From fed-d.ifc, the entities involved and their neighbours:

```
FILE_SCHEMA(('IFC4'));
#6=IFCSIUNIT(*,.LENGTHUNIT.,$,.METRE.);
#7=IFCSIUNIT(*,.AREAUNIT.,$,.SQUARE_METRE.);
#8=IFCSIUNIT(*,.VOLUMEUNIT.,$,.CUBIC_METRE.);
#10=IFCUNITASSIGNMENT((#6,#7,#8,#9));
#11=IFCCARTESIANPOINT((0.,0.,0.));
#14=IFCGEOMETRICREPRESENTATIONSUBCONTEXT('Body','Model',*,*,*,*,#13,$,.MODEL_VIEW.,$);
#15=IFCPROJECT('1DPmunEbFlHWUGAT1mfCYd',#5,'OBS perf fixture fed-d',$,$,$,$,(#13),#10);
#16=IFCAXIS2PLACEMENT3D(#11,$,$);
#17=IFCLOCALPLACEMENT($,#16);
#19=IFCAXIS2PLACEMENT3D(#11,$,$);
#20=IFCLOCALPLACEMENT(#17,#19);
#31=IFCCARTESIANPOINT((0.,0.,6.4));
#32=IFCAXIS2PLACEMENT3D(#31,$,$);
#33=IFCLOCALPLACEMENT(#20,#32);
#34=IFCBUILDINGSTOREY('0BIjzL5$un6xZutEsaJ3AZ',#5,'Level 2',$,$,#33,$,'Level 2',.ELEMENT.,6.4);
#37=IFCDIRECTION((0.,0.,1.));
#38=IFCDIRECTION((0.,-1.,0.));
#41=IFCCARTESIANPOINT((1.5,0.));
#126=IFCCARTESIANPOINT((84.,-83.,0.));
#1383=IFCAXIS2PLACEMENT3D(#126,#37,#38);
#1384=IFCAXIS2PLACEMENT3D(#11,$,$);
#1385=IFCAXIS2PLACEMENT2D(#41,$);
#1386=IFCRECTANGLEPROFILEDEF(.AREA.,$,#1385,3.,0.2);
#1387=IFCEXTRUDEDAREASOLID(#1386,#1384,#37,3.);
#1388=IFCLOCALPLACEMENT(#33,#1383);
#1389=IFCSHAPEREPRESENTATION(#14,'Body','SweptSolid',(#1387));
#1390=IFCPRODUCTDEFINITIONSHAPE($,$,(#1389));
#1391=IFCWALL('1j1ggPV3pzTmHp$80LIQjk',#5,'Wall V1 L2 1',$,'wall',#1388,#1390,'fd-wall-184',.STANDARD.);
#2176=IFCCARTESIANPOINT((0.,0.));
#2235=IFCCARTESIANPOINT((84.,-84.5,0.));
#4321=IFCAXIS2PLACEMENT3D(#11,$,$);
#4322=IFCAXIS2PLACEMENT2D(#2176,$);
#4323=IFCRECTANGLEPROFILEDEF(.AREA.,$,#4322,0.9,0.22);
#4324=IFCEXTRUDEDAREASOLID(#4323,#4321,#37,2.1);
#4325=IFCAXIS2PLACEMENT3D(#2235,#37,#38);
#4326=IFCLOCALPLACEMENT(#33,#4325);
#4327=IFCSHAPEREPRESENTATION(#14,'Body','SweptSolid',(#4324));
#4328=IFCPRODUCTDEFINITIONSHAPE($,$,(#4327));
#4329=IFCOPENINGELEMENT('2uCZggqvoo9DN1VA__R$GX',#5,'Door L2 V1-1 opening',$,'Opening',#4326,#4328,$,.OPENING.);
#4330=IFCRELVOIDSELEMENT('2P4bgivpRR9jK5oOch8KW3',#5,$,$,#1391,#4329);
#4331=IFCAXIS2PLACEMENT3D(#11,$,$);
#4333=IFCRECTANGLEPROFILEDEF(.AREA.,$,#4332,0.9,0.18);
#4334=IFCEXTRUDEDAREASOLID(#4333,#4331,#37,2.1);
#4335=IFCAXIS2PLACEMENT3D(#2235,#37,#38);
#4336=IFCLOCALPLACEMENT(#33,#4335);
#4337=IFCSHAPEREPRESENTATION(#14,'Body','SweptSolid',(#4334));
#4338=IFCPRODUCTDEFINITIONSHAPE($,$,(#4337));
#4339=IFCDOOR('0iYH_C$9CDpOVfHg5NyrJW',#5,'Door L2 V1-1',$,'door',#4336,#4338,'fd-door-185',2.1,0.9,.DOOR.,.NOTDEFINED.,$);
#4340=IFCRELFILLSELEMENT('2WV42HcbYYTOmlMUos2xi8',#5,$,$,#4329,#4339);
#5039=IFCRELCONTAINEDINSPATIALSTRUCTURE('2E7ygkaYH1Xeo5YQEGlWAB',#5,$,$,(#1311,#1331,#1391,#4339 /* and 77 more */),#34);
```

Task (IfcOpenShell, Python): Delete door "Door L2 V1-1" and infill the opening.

```python
import ifcopenshell
import ifcopenshell.api.feature
import ifcopenshell.api.root
import ifcopenshell.geom
import ifcopenshell.util.shape

model = ifcopenshell.open("fed-d.ifc")
settings = ifcopenshell.geom.settings()


def volume(element):
    """Net volume in cubic metres, openings subtracted."""
    shape = ifcopenshell.geom.create_shape(settings, element)
    return ifcopenshell.util.shape.get_volume(shape.geometry)


door = model.by_id(4339)
opening = door.FillsVoids[0].RelatingOpeningElement
wall = opening.VoidsElements[0].RelatingBuildingElement
before = volume(wall)

ifcopenshell.api.root.remove_product(model, product=door)
ifcopenshell.api.feature.remove_feature(model, feature=opening)

after = volume(wall)

print(f"wall volume {before:.3f} -> {after:.3f} m3")

model.write("fed-d_rev.ifc")
```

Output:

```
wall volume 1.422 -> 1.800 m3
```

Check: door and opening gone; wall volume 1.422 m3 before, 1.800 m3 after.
